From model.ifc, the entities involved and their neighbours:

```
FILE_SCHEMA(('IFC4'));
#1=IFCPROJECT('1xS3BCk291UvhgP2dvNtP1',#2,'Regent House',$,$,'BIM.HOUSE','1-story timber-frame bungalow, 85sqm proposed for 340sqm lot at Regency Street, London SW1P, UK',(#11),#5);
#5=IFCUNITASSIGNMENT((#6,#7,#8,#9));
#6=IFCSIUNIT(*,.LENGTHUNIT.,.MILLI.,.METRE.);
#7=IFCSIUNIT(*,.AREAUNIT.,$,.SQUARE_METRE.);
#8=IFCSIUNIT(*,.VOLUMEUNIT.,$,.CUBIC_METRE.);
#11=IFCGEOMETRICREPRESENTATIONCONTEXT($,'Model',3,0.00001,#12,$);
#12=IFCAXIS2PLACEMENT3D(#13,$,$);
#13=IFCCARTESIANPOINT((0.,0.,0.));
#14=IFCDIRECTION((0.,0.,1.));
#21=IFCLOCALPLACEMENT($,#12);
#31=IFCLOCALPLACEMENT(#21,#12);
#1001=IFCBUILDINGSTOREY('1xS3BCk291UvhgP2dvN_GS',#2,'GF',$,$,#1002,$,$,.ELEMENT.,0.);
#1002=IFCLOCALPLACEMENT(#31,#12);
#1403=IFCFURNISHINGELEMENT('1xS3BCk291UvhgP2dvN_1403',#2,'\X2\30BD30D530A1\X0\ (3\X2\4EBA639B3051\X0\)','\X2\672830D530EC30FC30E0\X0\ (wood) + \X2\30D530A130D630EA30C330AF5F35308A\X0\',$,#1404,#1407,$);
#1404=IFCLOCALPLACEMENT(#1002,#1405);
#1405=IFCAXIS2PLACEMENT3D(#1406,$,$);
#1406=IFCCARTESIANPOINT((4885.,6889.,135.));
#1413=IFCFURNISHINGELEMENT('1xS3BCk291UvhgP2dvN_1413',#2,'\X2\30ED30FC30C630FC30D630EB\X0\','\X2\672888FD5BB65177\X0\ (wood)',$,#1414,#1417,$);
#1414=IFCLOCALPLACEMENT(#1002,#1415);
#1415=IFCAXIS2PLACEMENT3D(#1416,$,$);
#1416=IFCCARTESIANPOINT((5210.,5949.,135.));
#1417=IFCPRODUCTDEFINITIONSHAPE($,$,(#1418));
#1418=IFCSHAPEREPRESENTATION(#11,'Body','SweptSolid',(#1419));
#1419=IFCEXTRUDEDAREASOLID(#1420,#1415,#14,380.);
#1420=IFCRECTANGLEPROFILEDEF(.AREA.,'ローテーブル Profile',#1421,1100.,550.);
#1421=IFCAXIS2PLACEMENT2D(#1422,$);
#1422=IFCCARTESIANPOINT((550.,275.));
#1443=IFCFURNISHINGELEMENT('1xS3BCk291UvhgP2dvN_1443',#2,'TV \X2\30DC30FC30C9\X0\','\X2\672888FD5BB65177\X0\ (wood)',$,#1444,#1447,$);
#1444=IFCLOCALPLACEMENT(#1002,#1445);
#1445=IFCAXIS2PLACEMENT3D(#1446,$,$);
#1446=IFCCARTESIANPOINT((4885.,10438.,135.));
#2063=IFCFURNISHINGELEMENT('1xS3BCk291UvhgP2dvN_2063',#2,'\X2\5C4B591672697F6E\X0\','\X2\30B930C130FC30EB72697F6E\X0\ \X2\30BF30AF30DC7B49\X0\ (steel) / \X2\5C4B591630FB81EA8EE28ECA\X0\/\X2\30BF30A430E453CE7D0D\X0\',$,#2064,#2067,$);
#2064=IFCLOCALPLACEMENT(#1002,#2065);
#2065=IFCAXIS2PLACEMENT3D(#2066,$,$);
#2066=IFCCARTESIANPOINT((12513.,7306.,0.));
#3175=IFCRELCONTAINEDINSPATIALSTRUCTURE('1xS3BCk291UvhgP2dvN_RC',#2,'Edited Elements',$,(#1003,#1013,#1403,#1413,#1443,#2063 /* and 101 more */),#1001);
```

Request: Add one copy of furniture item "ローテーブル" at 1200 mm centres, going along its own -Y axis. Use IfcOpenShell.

```python
import ifcopenshell
import ifcopenshell.api.geometry
import ifcopenshell.api.root
import ifcopenshell.util.element
import ifcopenshell.util.placement
import ifcopenshell.util.unit

model = ifcopenshell.open("model.ifc")
unit_scale = ifcopenshell.util.unit.calculate_unit_scale(model)


def reuse_history(source, copy):
    """copy_class also copies each property set's owner history, people and application; keep the originals."""
    for rel in copy.IsDefinedBy:
        if rel.is_a("IfcRelDefinesByProperties") and (history := rel.RelatingPropertyDefinition.OwnerHistory):
            rel.RelatingPropertyDefinition.OwnerHistory = source.OwnerHistory
            ifcopenshell.util.element.remove_deep2(model, history)


source = model.by_guid("1xS3BCk291UvhgP2dvN_1413")
base = ifcopenshell.util.placement.get_local_placement(source.ObjectPlacement)
step = -base[:3, 1] * 1.2 / unit_scale

for i in range(1, 2):
    copy = ifcopenshell.api.root.copy_class(model, product=source)
    copy.Representation = ifcopenshell.util.element.copy_deep(
        model, source.Representation, exclude=["IfcGeometricRepresentationContext", "IfcRepresentationMap"]
    )
    reuse_history(source, copy)
    matrix = base.copy()
    matrix[:3, 3] += i * step
    print("added at", matrix[:3, 3].round(3) + 0.0)
    ifcopenshell.api.geometry.edit_object_placement(model, product=copy, matrix=matrix, is_si=False)

model.write("model-out.ifc")
```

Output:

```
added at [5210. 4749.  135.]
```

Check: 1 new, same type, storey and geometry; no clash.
